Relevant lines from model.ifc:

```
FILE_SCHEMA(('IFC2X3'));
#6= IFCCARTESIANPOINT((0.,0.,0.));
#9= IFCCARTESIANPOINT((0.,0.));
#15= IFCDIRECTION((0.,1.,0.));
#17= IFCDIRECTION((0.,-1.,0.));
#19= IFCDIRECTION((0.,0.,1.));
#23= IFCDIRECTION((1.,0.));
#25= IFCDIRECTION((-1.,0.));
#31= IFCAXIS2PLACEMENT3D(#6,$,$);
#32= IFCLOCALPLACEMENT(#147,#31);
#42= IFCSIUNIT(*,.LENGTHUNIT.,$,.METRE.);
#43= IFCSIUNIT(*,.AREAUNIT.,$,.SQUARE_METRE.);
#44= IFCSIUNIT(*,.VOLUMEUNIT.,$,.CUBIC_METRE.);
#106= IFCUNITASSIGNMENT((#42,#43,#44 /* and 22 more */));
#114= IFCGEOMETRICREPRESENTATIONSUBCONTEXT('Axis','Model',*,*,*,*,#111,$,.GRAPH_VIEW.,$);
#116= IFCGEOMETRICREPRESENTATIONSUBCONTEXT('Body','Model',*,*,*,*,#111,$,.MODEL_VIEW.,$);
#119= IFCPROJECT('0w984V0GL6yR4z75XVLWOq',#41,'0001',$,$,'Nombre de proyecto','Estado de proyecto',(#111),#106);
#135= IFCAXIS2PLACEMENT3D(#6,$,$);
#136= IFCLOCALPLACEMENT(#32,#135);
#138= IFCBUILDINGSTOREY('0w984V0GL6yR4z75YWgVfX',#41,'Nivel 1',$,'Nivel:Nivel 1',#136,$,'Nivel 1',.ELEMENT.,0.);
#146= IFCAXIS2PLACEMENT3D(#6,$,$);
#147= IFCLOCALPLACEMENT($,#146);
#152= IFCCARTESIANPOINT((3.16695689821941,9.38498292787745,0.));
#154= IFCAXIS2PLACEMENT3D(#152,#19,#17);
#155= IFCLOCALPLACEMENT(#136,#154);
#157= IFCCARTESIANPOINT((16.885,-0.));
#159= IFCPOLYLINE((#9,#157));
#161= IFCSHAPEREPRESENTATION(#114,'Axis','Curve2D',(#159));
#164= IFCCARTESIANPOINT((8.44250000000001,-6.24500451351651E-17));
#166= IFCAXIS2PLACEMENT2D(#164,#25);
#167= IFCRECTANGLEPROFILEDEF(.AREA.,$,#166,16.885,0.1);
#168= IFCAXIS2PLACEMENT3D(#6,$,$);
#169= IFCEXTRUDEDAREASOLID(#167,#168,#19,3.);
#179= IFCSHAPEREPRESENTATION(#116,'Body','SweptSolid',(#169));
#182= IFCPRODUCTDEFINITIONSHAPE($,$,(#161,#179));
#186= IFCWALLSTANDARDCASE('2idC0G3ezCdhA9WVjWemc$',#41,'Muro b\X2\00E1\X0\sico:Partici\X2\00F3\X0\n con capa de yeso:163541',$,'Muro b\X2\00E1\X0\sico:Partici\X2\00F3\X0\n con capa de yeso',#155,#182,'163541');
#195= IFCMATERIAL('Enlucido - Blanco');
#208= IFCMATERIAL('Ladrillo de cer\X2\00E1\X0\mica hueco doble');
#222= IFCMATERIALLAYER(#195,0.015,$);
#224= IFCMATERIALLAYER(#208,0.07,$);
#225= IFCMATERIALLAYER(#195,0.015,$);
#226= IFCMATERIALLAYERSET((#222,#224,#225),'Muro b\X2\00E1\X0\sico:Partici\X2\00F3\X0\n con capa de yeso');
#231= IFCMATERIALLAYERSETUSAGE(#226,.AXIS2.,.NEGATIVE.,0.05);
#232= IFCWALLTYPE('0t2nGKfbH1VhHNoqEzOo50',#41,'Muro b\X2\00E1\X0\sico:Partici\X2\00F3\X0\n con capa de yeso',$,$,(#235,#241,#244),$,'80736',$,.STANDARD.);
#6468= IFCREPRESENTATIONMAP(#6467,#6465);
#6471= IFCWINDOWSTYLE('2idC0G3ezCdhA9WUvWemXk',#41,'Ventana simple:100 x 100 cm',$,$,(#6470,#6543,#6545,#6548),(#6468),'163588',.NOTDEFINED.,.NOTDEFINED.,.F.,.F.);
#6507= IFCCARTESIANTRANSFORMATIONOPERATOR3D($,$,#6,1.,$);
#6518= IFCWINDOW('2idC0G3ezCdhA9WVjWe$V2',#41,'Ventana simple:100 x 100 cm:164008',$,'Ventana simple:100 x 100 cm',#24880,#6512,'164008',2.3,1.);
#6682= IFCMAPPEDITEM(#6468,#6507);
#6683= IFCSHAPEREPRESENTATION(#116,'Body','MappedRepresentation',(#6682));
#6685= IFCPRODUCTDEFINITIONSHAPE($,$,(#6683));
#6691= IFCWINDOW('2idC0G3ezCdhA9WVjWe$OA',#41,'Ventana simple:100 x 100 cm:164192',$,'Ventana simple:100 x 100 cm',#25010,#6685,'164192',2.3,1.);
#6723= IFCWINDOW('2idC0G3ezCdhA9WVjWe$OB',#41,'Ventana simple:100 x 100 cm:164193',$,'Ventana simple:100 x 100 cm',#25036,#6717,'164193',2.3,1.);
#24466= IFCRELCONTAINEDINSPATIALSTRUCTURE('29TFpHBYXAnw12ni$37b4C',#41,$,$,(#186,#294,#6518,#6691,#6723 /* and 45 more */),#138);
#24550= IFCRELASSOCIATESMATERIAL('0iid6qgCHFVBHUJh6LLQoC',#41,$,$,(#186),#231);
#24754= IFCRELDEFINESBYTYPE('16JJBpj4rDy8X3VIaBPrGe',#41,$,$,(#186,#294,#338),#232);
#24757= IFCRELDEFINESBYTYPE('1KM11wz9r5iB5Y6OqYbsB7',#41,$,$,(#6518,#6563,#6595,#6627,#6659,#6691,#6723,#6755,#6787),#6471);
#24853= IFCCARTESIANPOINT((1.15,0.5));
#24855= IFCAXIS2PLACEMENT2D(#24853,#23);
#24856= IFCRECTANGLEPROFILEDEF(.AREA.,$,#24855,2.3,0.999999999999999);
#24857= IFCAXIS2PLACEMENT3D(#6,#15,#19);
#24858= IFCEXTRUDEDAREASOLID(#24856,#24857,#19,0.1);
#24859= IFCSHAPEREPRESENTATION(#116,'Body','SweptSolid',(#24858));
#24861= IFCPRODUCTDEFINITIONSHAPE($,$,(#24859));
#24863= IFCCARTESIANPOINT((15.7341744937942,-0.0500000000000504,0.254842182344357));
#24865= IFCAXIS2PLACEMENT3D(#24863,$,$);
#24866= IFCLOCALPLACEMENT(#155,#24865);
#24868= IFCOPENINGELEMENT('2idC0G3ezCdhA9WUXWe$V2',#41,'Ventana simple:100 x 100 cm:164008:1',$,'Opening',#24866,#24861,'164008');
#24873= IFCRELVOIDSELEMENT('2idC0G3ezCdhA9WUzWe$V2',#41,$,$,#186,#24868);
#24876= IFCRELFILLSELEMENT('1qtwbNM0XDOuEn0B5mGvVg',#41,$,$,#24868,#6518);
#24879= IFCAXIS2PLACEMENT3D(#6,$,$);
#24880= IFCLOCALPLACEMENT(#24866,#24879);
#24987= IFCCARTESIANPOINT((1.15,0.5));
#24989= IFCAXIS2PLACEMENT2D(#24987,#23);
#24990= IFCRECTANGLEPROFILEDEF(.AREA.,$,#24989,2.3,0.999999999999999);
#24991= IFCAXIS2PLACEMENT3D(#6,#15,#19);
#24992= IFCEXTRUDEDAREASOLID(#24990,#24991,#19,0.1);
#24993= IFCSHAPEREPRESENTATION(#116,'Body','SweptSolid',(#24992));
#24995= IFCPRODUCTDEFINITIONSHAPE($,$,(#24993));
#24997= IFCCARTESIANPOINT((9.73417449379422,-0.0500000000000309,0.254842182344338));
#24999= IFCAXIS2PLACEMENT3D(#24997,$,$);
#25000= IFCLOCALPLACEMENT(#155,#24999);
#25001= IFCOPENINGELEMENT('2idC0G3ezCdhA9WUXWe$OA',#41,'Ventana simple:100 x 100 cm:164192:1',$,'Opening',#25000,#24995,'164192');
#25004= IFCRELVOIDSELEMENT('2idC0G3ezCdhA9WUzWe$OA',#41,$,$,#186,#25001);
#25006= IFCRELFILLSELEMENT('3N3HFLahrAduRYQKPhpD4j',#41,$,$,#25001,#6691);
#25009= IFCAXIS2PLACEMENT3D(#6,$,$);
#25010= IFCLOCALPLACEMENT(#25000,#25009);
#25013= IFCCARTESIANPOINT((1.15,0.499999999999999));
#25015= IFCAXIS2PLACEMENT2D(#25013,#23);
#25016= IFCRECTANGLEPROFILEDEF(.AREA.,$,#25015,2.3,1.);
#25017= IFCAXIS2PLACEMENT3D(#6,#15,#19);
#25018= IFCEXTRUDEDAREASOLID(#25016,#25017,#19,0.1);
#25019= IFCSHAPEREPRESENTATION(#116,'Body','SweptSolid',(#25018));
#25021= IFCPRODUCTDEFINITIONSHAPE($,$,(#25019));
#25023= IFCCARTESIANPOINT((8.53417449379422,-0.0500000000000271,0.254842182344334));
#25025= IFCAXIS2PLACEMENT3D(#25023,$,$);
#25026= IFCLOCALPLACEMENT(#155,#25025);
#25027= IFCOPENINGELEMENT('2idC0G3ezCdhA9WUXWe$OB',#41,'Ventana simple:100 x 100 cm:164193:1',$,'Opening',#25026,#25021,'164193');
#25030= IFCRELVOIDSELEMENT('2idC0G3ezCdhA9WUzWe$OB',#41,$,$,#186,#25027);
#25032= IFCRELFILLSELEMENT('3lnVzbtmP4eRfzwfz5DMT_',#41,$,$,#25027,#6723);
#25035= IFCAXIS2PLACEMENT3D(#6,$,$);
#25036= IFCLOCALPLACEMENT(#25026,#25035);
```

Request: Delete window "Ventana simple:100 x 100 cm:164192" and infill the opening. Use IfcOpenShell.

```python
import ifcopenshell
import ifcopenshell.api.feature
import ifcopenshell.api.root
import ifcopenshell.geom
import ifcopenshell.util.shape

model = ifcopenshell.open("model.ifc")
settings = ifcopenshell.geom.settings()


def volume(element):
    """Net volume in cubic metres, openings subtracted."""
    shape = ifcopenshell.geom.create_shape(settings, element)
    return ifcopenshell.util.shape.get_volume(shape.geometry)


window = model.by_guid("2idC0G3ezCdhA9WVjWe$OA")
opening = window.FillsVoids[0].RelatingOpeningElement
wall = opening.VoidsElements[0].RelatingBuildingElement
before = volume(wall)

ifcopenshell.api.root.remove_product(model, product=window)
ifcopenshell.api.feature.remove_feature(model, feature=opening)

after = volume(wall)

print(f"wall volume {before:.3f} -> {after:.3f} m3")

model.write("model_rev.ifc")
```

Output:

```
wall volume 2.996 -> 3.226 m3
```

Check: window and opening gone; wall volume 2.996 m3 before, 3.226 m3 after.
